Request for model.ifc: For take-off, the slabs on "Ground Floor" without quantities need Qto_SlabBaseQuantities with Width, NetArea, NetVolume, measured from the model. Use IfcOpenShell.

First a look at what the model holds.

```python
import ifcopenshell
import ifcopenshell.util.element
import ifcopenshell.util.unit

model = ifcopenshell.open("model.ifc")
print(model.schema)
for unit_type in ("LENGTHUNIT", "AREAUNIT", "VOLUMEUNIT"):
    print(unit_type, ifcopenshell.util.unit.calculate_unit_scale(model, unit_type))
storey = next(s for s in model.by_type("IfcBuildingStorey") if s.Name == "Ground Floor")
slabs = [e for e in ifcopenshell.util.element.get_decomposition(storey) if e.is_a("IfcSlab")]
for e in sorted(slabs, key=lambda e: e.id()):
    print(e.id(), e.is_a(), e.Name, list(ifcopenshell.util.element.get_psets(e, qtos_only=True)), sep=" | ")
```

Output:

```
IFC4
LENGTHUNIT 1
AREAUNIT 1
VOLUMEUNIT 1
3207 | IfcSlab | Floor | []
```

```python
import ifcopenshell
import ifcopenshell.api.pset
import ifcopenshell.geom
import ifcopenshell.util.element
import ifcopenshell.util.shape
import ifcopenshell.util.unit

model = ifcopenshell.open("model.ifc")
unit_scale = ifcopenshell.util.unit.calculate_unit_scale(model)
area_scale = ifcopenshell.util.unit.calculate_unit_scale(model, "AREAUNIT")
volume_scale = ifcopenshell.util.unit.calculate_unit_scale(model, "VOLUMEUNIT")
settings = ifcopenshell.geom.settings()

storey = next(s for s in model.by_type("IfcBuildingStorey") if s.Name == "Ground Floor")
slabs = [e for e in ifcopenshell.util.element.get_decomposition(storey) if e.is_a("IfcSlab")]

for e in sorted(slabs, key=lambda e: e.id()):
    if ifcopenshell.util.element.get_psets(e, qtos_only=True, should_inherit=False):
        continue
    # Geometry comes back in metres, in the element's own axes.
    shape = ifcopenshell.geom.create_shape(settings, e)
    values = {
        "Width": ifcopenshell.util.shape.get_z(shape.geometry) / unit_scale,
        "NetArea": ifcopenshell.util.shape.get_footprint_area(shape.geometry) / area_scale,
        "NetVolume": ifcopenshell.util.shape.get_volume(shape.geometry) / volume_scale,
    }
    qto = ifcopenshell.api.pset.add_qto(model, product=e, name="Qto_SlabBaseQuantities")
    ifcopenshell.api.pset.edit_qto(model, qto=qto, properties=values)
    print(e.id(), {k: round(v, 3) for k, v in values.items()})

model.write("model_rev.ifc")
```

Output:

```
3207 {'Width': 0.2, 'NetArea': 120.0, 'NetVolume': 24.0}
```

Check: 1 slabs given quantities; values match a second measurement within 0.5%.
